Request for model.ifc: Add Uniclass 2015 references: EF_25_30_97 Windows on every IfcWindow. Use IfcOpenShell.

First a look at what the model holds.

```python
import ifcopenshell

model = ifcopenshell.open("model.ifc")
print(model.schema)
print("classifications:", [c.Name for c in model.by_type("IfcClassification")])
for ifc_class in ("IfcDoor", "IfcRoof", "IfcStair", "IfcWall", "IfcWindow"):
    print(ifc_class, len(model.by_type(ifc_class)))
```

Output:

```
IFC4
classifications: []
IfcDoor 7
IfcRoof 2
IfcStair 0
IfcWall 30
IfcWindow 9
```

```python
import ifcopenshell
import ifcopenshell.api.classification

model = ifcopenshell.open("model.ifc")

system = ifcopenshell.api.classification.add_classification(model, classification="Uniclass 2015")

codes = {
    "IfcWindow": ("EF_25_30_97", "Windows"),
}
for ifc_class, (code, name) in codes.items():
    products = model.by_type(ifc_class)
    ifcopenshell.api.classification.add_reference(
        model, products=products, classification=system, identification=code, name=name
    )
    print(code, len(products))

model.write("model_edited.ifc")
```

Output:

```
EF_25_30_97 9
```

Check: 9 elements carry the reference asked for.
